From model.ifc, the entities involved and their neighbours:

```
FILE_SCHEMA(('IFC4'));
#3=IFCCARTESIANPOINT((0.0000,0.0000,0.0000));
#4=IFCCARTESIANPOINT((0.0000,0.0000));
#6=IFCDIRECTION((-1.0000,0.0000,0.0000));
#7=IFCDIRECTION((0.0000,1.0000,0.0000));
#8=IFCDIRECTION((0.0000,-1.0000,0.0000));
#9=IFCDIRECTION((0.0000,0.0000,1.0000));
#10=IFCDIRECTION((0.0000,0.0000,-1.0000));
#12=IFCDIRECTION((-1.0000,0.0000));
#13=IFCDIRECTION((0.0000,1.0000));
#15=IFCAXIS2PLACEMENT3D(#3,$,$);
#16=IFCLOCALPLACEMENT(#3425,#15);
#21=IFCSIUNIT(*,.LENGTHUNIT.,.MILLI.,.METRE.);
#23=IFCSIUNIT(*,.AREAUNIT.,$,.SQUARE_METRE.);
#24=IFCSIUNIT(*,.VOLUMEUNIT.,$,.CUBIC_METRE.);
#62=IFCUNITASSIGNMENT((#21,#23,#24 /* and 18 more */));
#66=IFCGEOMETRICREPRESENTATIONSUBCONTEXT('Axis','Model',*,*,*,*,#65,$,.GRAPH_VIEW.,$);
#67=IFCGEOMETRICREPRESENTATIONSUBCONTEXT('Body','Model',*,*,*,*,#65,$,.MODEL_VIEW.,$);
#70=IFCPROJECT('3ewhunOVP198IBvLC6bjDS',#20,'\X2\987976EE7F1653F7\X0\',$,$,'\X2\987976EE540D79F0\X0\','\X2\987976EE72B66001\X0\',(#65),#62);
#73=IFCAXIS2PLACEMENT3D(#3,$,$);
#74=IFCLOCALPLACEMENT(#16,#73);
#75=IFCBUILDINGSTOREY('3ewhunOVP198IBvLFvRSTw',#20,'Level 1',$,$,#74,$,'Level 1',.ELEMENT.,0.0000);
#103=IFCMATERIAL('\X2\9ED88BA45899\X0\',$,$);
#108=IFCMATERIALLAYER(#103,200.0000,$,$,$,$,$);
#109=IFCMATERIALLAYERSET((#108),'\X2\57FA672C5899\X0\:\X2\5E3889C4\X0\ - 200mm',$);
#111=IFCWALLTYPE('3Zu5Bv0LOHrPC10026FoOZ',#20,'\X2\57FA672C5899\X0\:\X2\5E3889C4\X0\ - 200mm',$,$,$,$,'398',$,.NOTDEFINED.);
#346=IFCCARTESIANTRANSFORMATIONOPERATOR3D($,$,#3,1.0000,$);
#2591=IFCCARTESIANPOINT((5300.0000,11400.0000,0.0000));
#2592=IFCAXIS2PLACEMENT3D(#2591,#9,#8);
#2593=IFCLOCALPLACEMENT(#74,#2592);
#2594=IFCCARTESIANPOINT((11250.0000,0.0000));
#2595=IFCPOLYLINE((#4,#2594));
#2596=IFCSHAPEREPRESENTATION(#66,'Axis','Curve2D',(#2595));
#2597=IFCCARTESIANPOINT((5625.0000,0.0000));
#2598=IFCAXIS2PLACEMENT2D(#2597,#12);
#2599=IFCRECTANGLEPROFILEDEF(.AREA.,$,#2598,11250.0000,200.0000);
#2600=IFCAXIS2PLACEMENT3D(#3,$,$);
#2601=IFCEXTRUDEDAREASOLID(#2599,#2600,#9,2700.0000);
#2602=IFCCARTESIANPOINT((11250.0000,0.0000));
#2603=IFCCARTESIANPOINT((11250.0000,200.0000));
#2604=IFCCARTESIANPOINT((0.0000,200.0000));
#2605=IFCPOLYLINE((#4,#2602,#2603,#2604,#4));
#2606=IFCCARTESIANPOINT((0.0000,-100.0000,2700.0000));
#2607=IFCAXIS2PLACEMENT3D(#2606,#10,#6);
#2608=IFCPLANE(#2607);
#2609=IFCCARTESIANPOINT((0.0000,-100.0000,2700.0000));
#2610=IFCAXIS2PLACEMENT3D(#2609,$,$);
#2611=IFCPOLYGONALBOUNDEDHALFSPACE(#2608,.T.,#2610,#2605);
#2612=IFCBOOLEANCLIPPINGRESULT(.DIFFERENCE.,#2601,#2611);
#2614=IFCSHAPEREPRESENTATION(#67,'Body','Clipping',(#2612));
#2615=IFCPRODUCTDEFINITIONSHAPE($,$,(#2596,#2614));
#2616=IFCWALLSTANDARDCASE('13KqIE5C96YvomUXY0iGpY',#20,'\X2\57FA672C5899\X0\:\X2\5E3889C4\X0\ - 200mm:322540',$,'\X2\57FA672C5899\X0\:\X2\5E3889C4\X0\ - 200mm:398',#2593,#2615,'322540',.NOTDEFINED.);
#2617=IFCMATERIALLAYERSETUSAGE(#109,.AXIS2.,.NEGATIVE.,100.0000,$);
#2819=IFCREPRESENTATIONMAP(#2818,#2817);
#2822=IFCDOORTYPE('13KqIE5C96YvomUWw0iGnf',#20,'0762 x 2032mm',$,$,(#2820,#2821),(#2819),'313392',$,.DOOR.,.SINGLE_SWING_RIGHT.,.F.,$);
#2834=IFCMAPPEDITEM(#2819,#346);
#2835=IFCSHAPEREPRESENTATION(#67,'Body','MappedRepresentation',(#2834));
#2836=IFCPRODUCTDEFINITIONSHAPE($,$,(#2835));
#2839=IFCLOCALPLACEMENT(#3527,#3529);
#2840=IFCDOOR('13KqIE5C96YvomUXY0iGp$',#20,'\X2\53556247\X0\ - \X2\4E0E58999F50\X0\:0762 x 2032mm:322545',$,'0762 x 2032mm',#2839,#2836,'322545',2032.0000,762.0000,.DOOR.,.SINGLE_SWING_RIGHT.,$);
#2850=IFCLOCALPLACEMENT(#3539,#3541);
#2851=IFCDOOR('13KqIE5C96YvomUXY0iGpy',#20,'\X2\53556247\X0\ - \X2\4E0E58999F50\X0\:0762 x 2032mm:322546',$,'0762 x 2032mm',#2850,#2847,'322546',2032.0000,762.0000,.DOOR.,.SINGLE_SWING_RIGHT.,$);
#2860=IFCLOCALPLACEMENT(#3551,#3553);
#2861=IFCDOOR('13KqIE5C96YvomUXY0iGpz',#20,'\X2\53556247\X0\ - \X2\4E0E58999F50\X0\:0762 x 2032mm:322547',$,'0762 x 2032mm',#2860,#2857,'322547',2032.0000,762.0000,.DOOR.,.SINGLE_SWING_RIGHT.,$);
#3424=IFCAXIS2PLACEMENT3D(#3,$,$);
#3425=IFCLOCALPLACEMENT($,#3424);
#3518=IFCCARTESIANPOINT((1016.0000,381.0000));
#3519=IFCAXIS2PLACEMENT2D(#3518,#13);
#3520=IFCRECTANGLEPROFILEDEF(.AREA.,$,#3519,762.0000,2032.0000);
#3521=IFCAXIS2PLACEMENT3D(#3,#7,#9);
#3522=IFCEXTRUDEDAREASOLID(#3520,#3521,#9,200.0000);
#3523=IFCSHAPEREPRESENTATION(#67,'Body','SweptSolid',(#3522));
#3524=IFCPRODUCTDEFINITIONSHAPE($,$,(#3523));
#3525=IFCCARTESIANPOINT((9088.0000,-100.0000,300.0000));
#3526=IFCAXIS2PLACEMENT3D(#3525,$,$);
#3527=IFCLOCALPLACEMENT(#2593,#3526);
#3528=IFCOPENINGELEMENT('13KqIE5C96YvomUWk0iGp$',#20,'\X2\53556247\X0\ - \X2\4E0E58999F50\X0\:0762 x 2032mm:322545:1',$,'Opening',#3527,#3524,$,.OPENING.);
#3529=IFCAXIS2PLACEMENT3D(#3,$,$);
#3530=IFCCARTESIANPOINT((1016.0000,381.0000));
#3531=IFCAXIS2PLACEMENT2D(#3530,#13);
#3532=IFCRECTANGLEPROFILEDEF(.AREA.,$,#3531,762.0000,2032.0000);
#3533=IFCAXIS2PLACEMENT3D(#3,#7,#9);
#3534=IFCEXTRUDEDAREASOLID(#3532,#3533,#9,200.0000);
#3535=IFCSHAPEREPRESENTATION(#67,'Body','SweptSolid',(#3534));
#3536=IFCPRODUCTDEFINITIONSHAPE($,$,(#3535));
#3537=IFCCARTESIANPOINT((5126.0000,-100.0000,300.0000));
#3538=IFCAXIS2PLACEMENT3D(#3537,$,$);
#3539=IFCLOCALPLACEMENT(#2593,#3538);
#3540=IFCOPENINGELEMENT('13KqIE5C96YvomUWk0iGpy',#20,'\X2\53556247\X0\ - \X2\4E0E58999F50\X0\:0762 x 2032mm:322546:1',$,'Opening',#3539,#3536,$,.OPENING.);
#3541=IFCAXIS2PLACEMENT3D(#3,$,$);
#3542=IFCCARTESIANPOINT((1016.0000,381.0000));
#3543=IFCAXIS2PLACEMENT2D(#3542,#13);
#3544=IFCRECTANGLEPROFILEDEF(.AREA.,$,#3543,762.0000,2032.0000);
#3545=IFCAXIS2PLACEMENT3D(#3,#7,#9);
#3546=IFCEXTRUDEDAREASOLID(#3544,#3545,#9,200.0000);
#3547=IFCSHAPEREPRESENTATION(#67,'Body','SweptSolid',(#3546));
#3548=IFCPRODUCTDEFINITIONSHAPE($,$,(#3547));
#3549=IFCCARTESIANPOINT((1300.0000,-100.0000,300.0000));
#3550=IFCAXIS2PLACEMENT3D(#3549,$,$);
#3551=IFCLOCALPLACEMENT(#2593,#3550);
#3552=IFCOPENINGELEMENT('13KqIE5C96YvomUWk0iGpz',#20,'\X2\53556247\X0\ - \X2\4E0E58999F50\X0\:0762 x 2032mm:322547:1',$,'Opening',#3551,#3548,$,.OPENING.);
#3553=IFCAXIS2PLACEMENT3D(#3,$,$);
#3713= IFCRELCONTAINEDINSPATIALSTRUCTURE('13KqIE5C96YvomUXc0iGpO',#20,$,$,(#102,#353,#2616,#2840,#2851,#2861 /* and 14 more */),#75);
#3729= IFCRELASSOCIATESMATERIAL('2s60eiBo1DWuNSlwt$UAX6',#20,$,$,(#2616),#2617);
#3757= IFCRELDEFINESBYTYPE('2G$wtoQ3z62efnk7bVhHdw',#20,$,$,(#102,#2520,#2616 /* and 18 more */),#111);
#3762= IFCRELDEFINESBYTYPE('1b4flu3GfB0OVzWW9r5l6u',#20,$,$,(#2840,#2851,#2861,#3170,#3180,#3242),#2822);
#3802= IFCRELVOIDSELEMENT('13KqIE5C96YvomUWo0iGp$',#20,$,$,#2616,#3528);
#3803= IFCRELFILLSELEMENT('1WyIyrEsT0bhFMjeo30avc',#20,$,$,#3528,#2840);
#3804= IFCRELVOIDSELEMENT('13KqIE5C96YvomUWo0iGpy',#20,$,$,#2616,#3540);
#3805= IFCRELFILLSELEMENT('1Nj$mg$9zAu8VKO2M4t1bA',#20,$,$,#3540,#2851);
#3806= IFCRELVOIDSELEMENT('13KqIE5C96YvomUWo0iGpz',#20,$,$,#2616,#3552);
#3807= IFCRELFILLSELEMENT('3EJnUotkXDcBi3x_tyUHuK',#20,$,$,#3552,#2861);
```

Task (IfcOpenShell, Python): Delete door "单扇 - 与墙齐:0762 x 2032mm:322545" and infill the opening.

```python
import ifcopenshell
import ifcopenshell.api.feature
import ifcopenshell.api.root
import ifcopenshell.geom
import ifcopenshell.util.shape

model = ifcopenshell.open("model.ifc")
settings = ifcopenshell.geom.settings()


def volume(element):
    """Net volume in cubic metres, openings subtracted."""
    shape = ifcopenshell.geom.create_shape(settings, element)
    return ifcopenshell.util.shape.get_volume(shape.geometry)


door = model.by_guid("13KqIE5C96YvomUXY0iGp$")
opening = door.FillsVoids[0].RelatingOpeningElement
wall = opening.VoidsElements[0].RelatingBuildingElement
before = volume(wall)

ifcopenshell.api.root.remove_product(model, product=door)
ifcopenshell.api.feature.remove_feature(model, feature=opening)

after = volume(wall)

print(f"wall volume {before:.3f} -> {after:.3f} m3")

model.write("model_edited.ifc")
```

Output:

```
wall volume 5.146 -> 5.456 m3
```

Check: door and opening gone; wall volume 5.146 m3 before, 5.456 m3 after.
